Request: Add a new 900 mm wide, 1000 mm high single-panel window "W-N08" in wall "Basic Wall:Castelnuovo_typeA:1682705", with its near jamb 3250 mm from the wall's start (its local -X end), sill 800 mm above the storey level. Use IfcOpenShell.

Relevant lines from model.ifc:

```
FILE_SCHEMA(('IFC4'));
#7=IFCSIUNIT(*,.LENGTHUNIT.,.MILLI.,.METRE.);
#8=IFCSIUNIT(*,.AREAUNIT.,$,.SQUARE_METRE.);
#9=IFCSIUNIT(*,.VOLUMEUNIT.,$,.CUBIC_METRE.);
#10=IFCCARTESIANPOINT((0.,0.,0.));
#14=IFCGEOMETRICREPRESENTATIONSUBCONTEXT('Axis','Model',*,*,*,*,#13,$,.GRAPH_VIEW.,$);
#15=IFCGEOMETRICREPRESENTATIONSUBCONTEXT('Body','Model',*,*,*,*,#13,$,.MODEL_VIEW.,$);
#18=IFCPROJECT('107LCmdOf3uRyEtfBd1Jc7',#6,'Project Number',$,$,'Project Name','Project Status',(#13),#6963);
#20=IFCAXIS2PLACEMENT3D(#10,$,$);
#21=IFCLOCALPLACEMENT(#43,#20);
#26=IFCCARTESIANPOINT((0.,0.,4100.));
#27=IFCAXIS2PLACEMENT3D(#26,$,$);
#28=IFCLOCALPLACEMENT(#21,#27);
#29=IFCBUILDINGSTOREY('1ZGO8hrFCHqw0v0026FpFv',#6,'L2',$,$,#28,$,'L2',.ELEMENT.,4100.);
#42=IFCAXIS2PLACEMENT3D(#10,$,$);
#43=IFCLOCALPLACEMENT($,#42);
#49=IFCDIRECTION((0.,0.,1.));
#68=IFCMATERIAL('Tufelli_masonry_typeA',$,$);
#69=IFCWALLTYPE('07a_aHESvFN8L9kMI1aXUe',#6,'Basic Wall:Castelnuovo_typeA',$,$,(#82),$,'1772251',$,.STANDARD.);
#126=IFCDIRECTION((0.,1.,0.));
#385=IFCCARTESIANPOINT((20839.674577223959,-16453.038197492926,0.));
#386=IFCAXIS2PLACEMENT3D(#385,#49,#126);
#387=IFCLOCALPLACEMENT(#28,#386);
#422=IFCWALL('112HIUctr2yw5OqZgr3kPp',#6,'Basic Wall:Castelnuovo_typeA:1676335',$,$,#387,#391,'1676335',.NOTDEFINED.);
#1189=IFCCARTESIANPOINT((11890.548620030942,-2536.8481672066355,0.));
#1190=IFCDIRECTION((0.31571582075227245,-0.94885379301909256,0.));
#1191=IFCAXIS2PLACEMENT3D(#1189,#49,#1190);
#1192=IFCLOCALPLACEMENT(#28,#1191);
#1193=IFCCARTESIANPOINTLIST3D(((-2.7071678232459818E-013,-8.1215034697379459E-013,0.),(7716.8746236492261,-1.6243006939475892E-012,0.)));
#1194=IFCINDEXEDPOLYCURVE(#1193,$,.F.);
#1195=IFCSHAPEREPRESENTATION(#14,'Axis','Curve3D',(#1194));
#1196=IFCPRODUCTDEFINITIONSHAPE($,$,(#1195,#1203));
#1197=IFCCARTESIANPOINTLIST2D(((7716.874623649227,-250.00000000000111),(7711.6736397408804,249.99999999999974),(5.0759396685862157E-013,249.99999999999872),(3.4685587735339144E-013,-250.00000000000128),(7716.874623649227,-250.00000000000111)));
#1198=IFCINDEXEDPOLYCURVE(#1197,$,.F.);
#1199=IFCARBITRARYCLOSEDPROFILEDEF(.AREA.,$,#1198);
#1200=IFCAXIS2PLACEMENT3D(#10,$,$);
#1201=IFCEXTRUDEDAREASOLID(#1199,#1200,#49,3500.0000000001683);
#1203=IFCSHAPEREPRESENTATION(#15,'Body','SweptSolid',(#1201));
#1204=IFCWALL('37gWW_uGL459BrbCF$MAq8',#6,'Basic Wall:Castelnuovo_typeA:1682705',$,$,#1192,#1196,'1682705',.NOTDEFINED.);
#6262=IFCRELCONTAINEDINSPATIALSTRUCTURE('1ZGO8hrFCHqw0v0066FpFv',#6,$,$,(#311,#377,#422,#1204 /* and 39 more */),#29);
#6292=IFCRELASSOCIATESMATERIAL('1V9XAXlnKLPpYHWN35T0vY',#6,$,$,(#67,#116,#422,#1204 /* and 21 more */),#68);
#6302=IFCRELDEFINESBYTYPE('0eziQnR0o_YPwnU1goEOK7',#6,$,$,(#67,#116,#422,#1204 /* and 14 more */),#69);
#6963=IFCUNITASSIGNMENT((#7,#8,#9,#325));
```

```python
import numpy as np
import ifcopenshell
import ifcopenshell.api.feature
import ifcopenshell.api.geometry
import ifcopenshell.api.root
import ifcopenshell.api.spatial
import ifcopenshell.geom
import ifcopenshell.util.element
import ifcopenshell.util.placement
import ifcopenshell.util.representation
import ifcopenshell.util.shape
import ifcopenshell.util.unit

model = ifcopenshell.open("model.ifc")
unit_scale = ifcopenshell.util.unit.calculate_unit_scale(model)
settings = ifcopenshell.geom.settings()


def volume(element):
    """Net volume in cubic metres, openings subtracted."""
    shape = ifcopenshell.geom.create_shape(settings, element)
    return ifcopenshell.util.shape.get_volume(shape.geometry)


wall = model.by_guid("37gWW_uGL459BrbCF$MAq8")
storey = ifcopenshell.util.element.get_container(wall, ifc_class="IfcBuildingStorey")
context = ifcopenshell.util.representation.get_context(model, "Model", "Body", "MODEL_VIEW")
before = volume(wall)

width, height, from_end, sill = 0.9, 1, 3.25, 0.8  # metres

# The wall runs along its own X axis, and the end named is its -X end.
wall_shape = ifcopenshell.geom.create_shape(settings, wall)
x, y, z = ifcopenshell.util.shape.get_vertices(wall_shape.geometry).T
start = x.min() + from_end
face, thickness = float(y.min()), float(y.max() - y.min())
wall_matrix = ifcopenshell.util.placement.get_local_placement(wall.ObjectPlacement)
level = ifcopenshell.util.placement.get_local_placement(storey.ObjectPlacement)[2, 3]


def in_wall(x, y):
    """Placement at x, y metres in the wall's axes, at sill height."""
    matrix = wall_matrix.copy()
    matrix[:, 3] = wall_matrix @ np.array([x / unit_scale, y / unit_scale, 0.0, 1.0])
    matrix[2, 3] = level + sill / unit_scale
    return matrix


# Opening: a box that overshoots both wall faces by 50 mm.
opening = ifcopenshell.api.root.create_entity(model, ifc_class="IfcOpeningElement", predefined_type="OPENING")
box = ifcopenshell.api.geometry.add_wall_representation(
    model, context=context, length=width, height=height, thickness=thickness + 0.1
)
ifcopenshell.api.geometry.assign_representation(model, product=opening, representation=box)
ifcopenshell.api.geometry.edit_object_placement(model, product=opening, matrix=in_wall(start, face - 0.05), is_si=False)
ifcopenshell.api.feature.add_feature(model, feature=opening, element=wall)

window = ifcopenshell.api.root.create_entity(model, ifc_class="IfcWindow", name="W-N08", predefined_type="WINDOW")
window.OverallWidth, window.OverallHeight = width / unit_scale, height / unit_scale
window.PartitioningType = "SINGLE_PANEL"
body = ifcopenshell.api.geometry.add_window_representation(
    model,
    context=context,
    overall_width=window.OverallWidth,
    overall_height=window.OverallHeight,
    partition_type="SINGLE_PANEL",
)
ifcopenshell.api.geometry.assign_representation(model, product=window, representation=body)
ifcopenshell.api.spatial.assign_container(model, products=[window], relating_structure=storey)
ifcopenshell.api.feature.add_filling(model, opening=opening, element=window)

# Centre the window in the wall's thickness.
ifcopenshell.api.geometry.edit_object_placement(model, product=window, matrix=in_wall(start, face), is_si=False)
window_shape = ifcopenshell.geom.create_shape(settings, window)
depth = ifcopenshell.util.shape.get_vertices(window_shape.geometry)[:, 1]
offset = face + thickness / 2 - (depth.min() + depth.max()) / 2
ifcopenshell.api.geometry.edit_object_placement(model, product=window, matrix=in_wall(start, offset), is_si=False)

after = volume(wall)

print(f"wall volume {before:.3f} -> {after:.3f} m3")

model.write("model-out.ifc")
```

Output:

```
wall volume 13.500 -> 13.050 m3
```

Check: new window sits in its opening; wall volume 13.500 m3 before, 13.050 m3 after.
